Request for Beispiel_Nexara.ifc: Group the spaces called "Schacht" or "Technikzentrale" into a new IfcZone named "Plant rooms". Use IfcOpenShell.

First a look at what the model holds.

```python
import ifcopenshell

model = ifcopenshell.open("Beispiel_Nexara.ifc")
print(model.schema)
seen = {}
for space in model.by_type("IfcSpace"):
    seen[space.LongName] = seen.get(space.LongName, 0) + 1
for name, count in sorted(seen.items(), key=str):
    print(count, "x", name)
print("zones:", [z.Name for z in model.by_type("IfcZone")][:20])
```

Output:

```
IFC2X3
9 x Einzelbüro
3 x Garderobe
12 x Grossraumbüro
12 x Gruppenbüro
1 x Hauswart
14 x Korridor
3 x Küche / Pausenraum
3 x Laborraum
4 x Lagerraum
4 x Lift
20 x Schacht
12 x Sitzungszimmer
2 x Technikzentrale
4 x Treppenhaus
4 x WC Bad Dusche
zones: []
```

```python
import ifcopenshell
import ifcopenshell.api.group
import ifcopenshell.api.root

model = ifcopenshell.open("Beispiel_Nexara.ifc")

names = {"Schacht", "Technikzentrale"}
spaces = [s for s in model.by_type("IfcSpace") if s.LongName in names]

zone = ifcopenshell.api.root.create_entity(model, ifc_class="IfcZone", name="Plant rooms")
ifcopenshell.api.group.assign_group(model, products=spaces, group=zone)
print(len(spaces), "spaces in", zone.Name)

model.write("Beispiel_Nexara_rev.ifc")
```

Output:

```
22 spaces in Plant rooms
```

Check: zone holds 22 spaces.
